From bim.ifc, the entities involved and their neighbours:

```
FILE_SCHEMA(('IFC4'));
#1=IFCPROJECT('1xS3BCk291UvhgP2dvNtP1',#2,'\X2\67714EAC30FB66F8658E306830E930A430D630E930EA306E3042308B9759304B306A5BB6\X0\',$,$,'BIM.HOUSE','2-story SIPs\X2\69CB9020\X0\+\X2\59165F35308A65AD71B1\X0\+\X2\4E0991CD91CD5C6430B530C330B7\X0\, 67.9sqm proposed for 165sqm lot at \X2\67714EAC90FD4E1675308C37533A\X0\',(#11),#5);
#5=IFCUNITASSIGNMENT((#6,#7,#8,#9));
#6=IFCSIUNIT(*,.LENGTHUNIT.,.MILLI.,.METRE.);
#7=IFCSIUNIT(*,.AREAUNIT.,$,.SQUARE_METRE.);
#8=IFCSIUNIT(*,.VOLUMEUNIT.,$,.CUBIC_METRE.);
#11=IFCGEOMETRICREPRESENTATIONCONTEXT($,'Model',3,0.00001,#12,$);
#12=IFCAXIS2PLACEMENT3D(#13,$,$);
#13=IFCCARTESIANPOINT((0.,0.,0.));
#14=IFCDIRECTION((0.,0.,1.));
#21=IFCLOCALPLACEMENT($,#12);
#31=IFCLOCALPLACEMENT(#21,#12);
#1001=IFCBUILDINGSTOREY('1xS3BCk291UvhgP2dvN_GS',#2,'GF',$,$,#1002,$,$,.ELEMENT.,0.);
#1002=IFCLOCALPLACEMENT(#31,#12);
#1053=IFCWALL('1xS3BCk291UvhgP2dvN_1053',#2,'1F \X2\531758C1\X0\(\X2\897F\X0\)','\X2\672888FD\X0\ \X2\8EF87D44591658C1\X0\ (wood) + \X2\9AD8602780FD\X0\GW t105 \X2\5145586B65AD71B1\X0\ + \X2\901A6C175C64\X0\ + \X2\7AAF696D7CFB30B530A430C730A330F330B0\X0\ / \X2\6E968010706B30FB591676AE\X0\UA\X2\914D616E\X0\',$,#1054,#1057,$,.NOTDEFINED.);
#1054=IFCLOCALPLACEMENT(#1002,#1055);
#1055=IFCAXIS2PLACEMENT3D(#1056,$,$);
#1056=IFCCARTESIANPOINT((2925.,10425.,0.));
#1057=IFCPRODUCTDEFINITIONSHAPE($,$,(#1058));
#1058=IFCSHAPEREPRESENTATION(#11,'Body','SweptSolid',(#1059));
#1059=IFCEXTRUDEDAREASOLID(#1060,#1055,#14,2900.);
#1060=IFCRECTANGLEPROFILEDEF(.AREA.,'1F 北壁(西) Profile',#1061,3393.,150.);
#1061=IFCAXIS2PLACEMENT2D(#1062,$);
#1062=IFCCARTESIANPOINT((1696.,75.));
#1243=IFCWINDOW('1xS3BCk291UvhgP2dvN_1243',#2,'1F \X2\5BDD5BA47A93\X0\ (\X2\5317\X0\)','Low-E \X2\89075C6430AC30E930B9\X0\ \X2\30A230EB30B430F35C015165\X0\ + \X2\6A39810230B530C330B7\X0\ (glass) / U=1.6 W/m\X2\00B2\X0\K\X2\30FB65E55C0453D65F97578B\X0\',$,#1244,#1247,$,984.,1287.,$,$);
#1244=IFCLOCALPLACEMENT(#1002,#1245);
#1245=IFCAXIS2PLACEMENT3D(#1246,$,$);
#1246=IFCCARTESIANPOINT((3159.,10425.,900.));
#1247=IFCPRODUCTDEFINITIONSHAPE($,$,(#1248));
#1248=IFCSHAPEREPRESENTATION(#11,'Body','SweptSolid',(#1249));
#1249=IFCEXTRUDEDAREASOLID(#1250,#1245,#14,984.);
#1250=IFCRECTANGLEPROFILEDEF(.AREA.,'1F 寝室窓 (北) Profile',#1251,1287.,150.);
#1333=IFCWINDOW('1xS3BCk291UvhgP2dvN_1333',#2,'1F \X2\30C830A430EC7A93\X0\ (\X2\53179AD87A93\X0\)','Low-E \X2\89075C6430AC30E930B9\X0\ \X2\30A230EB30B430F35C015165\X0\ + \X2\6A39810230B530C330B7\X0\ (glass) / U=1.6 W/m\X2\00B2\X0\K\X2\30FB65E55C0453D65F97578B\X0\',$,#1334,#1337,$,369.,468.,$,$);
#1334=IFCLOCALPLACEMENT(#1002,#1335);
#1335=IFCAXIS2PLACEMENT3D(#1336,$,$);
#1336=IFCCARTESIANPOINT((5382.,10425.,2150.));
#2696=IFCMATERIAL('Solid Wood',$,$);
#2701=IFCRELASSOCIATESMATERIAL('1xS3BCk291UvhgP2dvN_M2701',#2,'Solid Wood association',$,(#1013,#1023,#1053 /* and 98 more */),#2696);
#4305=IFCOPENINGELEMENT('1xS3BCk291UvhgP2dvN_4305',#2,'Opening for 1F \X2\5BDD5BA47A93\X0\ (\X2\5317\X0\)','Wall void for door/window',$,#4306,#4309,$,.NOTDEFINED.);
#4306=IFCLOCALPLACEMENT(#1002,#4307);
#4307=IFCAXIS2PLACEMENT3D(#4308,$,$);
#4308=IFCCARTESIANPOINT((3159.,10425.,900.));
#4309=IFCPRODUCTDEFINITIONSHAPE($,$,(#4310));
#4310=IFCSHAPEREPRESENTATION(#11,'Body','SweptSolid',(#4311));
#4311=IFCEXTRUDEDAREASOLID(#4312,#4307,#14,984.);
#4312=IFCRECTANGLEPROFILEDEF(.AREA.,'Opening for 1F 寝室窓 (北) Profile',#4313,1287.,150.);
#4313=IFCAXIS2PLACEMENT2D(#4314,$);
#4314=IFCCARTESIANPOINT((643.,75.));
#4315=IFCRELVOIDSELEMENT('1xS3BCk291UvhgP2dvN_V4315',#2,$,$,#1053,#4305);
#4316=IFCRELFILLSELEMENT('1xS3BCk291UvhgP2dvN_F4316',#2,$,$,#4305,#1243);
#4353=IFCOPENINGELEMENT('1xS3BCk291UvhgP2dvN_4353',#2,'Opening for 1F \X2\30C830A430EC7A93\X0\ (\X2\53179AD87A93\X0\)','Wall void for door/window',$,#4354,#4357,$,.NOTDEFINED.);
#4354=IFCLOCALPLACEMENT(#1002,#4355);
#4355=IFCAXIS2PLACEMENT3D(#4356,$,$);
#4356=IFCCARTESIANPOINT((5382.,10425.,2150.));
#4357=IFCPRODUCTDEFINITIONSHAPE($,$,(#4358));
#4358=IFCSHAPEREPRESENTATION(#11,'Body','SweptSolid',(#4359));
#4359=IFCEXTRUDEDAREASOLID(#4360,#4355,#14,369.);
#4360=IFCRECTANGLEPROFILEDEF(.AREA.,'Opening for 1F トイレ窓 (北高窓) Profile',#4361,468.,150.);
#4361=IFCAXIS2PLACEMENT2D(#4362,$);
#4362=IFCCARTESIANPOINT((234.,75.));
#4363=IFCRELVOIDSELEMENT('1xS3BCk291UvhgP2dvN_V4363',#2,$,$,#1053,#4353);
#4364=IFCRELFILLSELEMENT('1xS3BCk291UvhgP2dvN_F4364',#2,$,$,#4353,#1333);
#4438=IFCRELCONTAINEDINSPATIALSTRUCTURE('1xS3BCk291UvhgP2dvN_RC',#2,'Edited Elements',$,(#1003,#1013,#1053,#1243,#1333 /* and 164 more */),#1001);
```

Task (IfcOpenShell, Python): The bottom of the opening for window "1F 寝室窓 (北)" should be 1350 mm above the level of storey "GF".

```python
import numpy as np
import ifcopenshell
import ifcopenshell.api.geometry
import ifcopenshell.geom
import ifcopenshell.util.element
import ifcopenshell.util.placement
import ifcopenshell.util.shape
import ifcopenshell.util.unit

model = ifcopenshell.open("bim.ifc")
unit_scale = ifcopenshell.util.unit.calculate_unit_scale(model)

window = model.by_guid("1xS3BCk291UvhgP2dvN_1243")
opening = window.FillsVoids[0].RelatingOpeningElement
storey = ifcopenshell.util.element.get_container(window, ifc_class="IfcBuildingStorey")
level = ifcopenshell.util.placement.get_local_placement(storey.ObjectPlacement)[2, 3]

# The opening's origin need not be at the sill, so measure its lowest point.
shape = ifcopenshell.geom.create_shape(ifcopenshell.geom.settings(), opening)
bottom = ifcopenshell.util.shape.get_shape_bottom_elevation(shape, shape.geometry) / unit_scale
dz = level + 1.35 / unit_scale - bottom

shift = np.array([0.0, 0.0, dz])
# The window is not placed relative to its opening, so move both.
for product in (opening, window):
    matrix = ifcopenshell.util.placement.get_local_placement(product.ObjectPlacement)
    matrix[:3, 3] += shift
    ifcopenshell.api.geometry.edit_object_placement(model, product=product, matrix=matrix, is_si=False)

print(f"moved by {dz * unit_scale:+.3f} m")

model.write("bim-out.ifc")
```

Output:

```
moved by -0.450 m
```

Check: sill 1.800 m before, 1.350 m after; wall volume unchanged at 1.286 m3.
